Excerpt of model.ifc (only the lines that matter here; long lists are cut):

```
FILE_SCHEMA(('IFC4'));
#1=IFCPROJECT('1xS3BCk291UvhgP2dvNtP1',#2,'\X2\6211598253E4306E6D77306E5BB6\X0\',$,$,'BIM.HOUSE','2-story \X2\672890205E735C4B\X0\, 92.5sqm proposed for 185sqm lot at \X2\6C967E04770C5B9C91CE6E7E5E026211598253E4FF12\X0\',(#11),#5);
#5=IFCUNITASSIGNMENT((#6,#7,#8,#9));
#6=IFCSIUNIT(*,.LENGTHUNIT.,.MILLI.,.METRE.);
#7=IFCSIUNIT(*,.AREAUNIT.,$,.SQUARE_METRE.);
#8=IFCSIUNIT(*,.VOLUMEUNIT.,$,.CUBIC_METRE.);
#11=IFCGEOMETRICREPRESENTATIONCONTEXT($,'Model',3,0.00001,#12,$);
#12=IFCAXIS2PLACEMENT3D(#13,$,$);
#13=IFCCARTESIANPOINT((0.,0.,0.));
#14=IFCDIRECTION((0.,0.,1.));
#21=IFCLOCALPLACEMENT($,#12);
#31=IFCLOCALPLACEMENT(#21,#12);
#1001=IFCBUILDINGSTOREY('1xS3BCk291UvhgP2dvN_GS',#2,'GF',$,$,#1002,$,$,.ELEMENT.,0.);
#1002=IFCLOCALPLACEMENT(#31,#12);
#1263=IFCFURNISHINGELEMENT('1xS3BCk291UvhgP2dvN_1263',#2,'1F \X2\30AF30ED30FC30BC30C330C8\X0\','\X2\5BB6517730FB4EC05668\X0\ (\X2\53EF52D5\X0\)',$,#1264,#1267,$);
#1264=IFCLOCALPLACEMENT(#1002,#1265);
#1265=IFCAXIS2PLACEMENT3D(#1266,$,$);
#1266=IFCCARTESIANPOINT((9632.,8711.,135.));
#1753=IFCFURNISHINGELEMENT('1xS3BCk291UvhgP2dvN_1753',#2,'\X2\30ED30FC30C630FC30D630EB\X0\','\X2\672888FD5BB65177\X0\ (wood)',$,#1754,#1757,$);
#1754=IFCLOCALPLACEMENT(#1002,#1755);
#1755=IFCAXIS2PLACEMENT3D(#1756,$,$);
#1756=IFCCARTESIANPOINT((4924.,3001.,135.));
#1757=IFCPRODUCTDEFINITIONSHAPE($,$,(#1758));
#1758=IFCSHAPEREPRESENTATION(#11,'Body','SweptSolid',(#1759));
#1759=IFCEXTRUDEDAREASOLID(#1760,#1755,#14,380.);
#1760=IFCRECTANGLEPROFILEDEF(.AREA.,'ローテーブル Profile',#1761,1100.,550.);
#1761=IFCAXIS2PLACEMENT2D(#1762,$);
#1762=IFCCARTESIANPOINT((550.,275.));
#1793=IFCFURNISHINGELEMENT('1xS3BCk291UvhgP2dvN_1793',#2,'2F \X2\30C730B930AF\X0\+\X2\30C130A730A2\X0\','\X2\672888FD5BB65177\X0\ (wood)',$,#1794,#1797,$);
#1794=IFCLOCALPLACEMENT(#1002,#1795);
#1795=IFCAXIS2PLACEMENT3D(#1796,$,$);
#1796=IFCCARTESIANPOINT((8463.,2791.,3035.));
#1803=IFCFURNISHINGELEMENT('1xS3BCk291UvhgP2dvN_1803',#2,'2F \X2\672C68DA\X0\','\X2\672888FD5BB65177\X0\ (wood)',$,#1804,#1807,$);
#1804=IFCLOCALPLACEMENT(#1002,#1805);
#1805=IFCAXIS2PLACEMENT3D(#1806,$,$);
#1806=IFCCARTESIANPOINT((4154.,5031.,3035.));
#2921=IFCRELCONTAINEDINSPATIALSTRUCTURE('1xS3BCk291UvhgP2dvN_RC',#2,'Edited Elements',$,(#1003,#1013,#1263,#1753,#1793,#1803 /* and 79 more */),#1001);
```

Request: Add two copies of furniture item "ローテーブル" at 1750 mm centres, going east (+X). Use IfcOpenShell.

```python
import numpy as np
import ifcopenshell
import ifcopenshell.api.geometry
import ifcopenshell.api.root
import ifcopenshell.util.element
import ifcopenshell.util.placement
import ifcopenshell.util.unit

model = ifcopenshell.open("model.ifc")
unit_scale = ifcopenshell.util.unit.calculate_unit_scale(model)


def reuse_history(source, copy):
    """copy_class also copies each property set's owner history, people and application; keep the originals."""
    for rel in copy.IsDefinedBy:
        if rel.is_a("IfcRelDefinesByProperties") and (history := rel.RelatingPropertyDefinition.OwnerHistory):
            rel.RelatingPropertyDefinition.OwnerHistory = source.OwnerHistory
            ifcopenshell.util.element.remove_deep2(model, history)


source = model.by_id(1753)
base = ifcopenshell.util.placement.get_local_placement(source.ObjectPlacement)
step = np.array([1.0, 0.0, 0.0]) * 1.75 / unit_scale

for i in range(1, 3):
    copy = ifcopenshell.api.root.copy_class(model, product=source)
    copy.Representation = ifcopenshell.util.element.copy_deep(
        model, source.Representation, exclude=["IfcGeometricRepresentationContext", "IfcRepresentationMap"]
    )
    reuse_history(source, copy)
    matrix = base.copy()
    matrix[:3, 3] += i * step
    print("added at", matrix[:3, 3].round(3) + 0.0)
    ifcopenshell.api.geometry.edit_object_placement(model, product=copy, matrix=matrix, is_si=False)

model.write("model_edited.ifc")
```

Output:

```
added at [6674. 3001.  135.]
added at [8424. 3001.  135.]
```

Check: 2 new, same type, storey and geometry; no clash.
